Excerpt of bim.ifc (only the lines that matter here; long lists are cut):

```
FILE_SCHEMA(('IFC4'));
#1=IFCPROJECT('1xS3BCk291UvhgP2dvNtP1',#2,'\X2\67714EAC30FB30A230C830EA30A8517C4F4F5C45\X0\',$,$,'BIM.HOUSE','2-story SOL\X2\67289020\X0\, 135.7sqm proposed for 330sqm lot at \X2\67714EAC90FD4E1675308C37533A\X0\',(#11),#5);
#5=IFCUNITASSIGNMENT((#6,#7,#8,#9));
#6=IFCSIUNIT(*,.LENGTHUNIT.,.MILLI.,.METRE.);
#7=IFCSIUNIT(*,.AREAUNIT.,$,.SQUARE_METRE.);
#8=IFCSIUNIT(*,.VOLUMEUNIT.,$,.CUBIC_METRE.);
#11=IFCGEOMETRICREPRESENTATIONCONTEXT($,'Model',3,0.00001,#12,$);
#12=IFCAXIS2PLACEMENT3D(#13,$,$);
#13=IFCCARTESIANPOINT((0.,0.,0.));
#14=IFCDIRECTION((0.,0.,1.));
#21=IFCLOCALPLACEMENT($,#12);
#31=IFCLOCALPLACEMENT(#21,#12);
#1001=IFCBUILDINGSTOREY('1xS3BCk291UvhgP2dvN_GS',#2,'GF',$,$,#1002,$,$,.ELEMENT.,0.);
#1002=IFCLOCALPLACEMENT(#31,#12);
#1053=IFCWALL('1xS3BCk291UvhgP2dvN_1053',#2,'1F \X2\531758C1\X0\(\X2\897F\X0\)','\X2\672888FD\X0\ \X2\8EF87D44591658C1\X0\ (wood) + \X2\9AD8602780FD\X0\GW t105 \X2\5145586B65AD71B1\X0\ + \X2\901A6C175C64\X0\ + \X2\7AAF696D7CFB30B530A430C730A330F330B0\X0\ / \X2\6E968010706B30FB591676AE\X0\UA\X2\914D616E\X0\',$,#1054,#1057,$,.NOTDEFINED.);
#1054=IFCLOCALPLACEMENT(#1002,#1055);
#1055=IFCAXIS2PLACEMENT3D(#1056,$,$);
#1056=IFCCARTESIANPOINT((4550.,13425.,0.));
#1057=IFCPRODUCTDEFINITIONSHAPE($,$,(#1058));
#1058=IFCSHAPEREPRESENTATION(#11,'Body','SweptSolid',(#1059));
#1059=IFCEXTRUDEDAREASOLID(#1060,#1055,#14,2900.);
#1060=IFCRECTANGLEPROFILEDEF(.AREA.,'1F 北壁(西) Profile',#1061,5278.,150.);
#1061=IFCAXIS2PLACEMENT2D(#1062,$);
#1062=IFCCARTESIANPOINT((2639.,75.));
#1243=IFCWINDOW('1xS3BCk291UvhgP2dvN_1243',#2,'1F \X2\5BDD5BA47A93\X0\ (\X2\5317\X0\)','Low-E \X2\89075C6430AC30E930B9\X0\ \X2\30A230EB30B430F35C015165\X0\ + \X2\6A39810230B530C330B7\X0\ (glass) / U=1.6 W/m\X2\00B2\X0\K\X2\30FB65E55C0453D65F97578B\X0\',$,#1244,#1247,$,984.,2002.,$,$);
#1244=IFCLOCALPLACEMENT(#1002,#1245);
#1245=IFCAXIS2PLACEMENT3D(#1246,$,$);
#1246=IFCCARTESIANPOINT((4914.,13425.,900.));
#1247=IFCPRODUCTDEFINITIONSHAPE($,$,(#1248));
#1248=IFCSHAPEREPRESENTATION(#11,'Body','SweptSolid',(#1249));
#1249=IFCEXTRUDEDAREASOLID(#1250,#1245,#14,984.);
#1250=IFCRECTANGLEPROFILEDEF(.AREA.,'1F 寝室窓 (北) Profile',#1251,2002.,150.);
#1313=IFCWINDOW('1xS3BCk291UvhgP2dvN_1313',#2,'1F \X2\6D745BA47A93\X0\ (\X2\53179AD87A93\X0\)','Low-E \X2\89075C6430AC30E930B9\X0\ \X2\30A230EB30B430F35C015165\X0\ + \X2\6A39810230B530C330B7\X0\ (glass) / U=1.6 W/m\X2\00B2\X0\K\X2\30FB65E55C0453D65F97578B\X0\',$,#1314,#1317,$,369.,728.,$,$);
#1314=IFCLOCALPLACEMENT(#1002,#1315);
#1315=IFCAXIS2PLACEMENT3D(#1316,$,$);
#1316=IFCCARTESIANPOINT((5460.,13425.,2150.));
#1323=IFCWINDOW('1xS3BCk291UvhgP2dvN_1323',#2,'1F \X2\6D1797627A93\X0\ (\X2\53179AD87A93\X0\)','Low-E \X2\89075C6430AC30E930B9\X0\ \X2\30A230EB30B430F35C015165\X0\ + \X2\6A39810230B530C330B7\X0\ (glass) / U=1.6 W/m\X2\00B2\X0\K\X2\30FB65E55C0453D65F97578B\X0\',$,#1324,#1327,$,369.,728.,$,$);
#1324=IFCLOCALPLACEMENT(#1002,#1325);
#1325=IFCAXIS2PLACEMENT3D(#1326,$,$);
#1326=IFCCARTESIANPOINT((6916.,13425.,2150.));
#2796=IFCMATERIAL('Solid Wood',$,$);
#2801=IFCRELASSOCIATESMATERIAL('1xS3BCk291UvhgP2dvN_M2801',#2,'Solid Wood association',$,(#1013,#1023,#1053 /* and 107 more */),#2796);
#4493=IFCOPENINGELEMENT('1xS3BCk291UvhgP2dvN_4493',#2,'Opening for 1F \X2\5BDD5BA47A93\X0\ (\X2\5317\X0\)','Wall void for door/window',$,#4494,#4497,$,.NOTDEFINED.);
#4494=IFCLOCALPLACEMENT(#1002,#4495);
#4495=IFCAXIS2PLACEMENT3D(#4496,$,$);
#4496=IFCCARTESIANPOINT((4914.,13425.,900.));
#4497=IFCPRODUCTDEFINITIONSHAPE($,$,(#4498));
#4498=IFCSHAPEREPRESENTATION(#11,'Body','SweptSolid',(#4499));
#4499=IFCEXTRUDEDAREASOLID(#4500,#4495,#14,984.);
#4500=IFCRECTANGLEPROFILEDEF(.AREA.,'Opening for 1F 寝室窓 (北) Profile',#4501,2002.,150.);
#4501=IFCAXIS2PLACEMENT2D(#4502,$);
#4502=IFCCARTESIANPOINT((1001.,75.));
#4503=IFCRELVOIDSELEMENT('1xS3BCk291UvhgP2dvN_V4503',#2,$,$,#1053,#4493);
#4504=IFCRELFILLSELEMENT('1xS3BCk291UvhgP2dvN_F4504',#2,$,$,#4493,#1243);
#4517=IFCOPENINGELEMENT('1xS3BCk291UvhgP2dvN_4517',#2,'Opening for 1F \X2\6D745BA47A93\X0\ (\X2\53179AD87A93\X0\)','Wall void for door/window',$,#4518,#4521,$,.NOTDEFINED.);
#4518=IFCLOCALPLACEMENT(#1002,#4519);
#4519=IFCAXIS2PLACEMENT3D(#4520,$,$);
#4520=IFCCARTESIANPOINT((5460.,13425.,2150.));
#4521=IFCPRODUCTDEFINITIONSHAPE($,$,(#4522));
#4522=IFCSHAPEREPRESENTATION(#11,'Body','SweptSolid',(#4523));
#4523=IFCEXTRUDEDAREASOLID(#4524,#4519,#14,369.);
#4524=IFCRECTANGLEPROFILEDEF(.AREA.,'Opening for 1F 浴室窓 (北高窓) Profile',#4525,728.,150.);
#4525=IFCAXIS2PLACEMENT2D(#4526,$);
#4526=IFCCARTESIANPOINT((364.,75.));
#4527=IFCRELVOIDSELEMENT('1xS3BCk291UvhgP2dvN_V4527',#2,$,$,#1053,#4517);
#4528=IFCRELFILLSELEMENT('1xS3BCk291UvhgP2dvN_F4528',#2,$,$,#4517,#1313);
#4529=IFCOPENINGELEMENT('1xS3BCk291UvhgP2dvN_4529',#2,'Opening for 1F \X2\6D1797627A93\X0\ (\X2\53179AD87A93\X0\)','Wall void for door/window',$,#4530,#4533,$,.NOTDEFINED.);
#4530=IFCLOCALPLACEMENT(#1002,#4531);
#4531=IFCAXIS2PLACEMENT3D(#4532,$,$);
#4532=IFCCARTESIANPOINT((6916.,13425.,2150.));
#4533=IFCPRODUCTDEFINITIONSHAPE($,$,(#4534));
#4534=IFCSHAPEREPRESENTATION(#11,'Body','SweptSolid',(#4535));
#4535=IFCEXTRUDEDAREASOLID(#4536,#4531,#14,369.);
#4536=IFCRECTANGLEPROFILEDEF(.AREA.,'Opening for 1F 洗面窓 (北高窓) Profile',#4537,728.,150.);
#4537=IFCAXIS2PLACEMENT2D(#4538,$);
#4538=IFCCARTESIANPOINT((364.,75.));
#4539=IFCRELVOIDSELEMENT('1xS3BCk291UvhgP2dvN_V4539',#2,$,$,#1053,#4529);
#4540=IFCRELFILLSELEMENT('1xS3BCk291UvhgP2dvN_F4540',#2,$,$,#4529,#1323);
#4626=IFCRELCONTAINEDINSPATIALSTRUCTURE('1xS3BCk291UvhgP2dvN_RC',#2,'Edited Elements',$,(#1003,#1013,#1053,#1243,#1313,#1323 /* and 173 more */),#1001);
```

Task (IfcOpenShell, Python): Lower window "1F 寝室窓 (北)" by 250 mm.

```python
import numpy as np
import ifcopenshell
import ifcopenshell.api.geometry
import ifcopenshell.util.placement
import ifcopenshell.util.unit

model = ifcopenshell.open("bim.ifc")
unit_scale = ifcopenshell.util.unit.calculate_unit_scale(model)

window = model.by_guid("1xS3BCk291UvhgP2dvN_1243")
opening = window.FillsVoids[0].RelatingOpeningElement
dz = -0.25 / unit_scale

shift = np.array([0.0, 0.0, dz])
# The window is not placed relative to its opening, so move both.
for product in (opening, window):
    matrix = ifcopenshell.util.placement.get_local_placement(product.ObjectPlacement)
    matrix[:3, 3] += shift
    ifcopenshell.api.geometry.edit_object_placement(model, product=product, matrix=matrix, is_si=False)

print(f"moved by {dz * unit_scale:+.3f} m")

model.write("bim-out.ifc")
```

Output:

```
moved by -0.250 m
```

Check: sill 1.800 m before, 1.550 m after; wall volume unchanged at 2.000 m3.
